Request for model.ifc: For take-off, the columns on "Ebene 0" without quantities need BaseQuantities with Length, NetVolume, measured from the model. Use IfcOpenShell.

First a look at what the model holds.

```python
import ifcopenshell
import ifcopenshell.util.element
import ifcopenshell.util.unit

model = ifcopenshell.open("model.ifc")
print(model.schema)
for unit_type in ("LENGTHUNIT", "AREAUNIT", "VOLUMEUNIT"):
    print(unit_type, ifcopenshell.util.unit.calculate_unit_scale(model, unit_type))
storey = next(s for s in model.by_type("IfcBuildingStorey") if s.Name == "Ebene 0")
columns = [e for e in ifcopenshell.util.element.get_decomposition(storey) if e.is_a("IfcColumn")]
for e in sorted(columns, key=lambda e: e.id()):
    print(e.id(), e.is_a(), e.Name, list(ifcopenshell.util.element.get_psets(e, qtos_only=True)), sep=" | ")
```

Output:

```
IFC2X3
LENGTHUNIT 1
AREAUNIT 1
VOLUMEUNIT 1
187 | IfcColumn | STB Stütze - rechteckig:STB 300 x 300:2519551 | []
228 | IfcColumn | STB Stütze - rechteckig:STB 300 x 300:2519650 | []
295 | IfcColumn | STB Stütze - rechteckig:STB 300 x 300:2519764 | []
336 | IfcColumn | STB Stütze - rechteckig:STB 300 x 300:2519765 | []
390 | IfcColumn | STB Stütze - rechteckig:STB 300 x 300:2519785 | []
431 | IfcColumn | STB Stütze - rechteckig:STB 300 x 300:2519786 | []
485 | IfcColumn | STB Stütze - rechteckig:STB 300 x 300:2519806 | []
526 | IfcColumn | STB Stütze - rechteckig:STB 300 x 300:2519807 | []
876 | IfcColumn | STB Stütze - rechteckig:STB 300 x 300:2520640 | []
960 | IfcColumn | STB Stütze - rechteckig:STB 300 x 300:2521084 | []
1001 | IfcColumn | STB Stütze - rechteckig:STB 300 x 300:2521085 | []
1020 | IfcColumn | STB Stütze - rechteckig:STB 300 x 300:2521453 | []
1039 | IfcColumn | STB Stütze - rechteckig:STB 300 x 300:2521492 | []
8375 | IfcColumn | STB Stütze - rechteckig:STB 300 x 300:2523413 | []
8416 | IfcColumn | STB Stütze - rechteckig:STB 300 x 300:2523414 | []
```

```python
import ifcopenshell
import ifcopenshell.api.pset
import ifcopenshell.geom
import ifcopenshell.util.element
import ifcopenshell.util.shape
import ifcopenshell.util.unit

model = ifcopenshell.open("model.ifc")
unit_scale = ifcopenshell.util.unit.calculate_unit_scale(model)
volume_scale = ifcopenshell.util.unit.calculate_unit_scale(model, "VOLUMEUNIT")
settings = ifcopenshell.geom.settings()

storey = next(s for s in model.by_type("IfcBuildingStorey") if s.Name == "Ebene 0")
columns = [e for e in ifcopenshell.util.element.get_decomposition(storey) if e.is_a("IfcColumn")]

for e in sorted(columns, key=lambda e: e.id()):
    if ifcopenshell.util.element.get_psets(e, qtos_only=True, should_inherit=False):
        continue
    # Geometry comes back in metres, in the element's own axes.
    shape = ifcopenshell.geom.create_shape(settings, e)
    values = {
        "Length": ifcopenshell.util.shape.get_z(shape.geometry) / unit_scale,
        "NetVolume": ifcopenshell.util.shape.get_volume(shape.geometry) / volume_scale,
    }
    qto = ifcopenshell.api.pset.add_qto(model, product=e, name="BaseQuantities")
    ifcopenshell.api.pset.edit_qto(model, qto=qto, properties=values)
    print(e.id(), {k: round(v, 3) for k, v in values.items()})

model.write("model-out.ifc")
```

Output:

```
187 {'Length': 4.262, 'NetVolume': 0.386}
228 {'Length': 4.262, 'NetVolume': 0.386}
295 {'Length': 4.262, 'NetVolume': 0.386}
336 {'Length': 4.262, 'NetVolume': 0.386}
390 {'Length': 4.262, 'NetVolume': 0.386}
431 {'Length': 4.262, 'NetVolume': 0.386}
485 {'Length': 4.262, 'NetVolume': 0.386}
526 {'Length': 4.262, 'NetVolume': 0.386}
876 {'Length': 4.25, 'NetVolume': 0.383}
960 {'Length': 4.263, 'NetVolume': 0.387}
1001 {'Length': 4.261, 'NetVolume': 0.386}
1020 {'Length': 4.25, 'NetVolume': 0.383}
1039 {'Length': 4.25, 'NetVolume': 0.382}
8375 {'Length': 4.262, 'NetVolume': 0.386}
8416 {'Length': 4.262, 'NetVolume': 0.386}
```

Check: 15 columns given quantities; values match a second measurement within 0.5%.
